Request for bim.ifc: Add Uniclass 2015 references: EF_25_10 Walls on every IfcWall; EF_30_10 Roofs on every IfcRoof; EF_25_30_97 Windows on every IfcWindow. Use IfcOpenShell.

First a look at what the model holds.

```python
import ifcopenshell

model = ifcopenshell.open("bim.ifc")
print(model.schema)
print("classifications:", [c.Name for c in model.by_type("IfcClassification")])
for ifc_class in ("IfcDoor", "IfcRoof", "IfcStair", "IfcWall", "IfcWindow"):
    print(ifc_class, len(model.by_type(ifc_class)))
```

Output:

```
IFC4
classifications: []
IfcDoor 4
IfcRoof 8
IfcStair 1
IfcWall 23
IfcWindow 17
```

```python
import ifcopenshell
import ifcopenshell.api.classification

model = ifcopenshell.open("bim.ifc")

system = ifcopenshell.api.classification.add_classification(model, classification="Uniclass 2015")

codes = {
    "IfcWall": ("EF_25_10", "Walls"),
    "IfcRoof": ("EF_30_10", "Roofs"),
    "IfcWindow": ("EF_25_30_97", "Windows"),
}
for ifc_class, (code, name) in codes.items():
    products = model.by_type(ifc_class)
    ifcopenshell.api.classification.add_reference(
        model, products=products, classification=system, identification=code, name=name
    )
    print(code, len(products))

model.write("bim_updated.ifc")
```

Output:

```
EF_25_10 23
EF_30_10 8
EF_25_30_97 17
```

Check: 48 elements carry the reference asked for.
